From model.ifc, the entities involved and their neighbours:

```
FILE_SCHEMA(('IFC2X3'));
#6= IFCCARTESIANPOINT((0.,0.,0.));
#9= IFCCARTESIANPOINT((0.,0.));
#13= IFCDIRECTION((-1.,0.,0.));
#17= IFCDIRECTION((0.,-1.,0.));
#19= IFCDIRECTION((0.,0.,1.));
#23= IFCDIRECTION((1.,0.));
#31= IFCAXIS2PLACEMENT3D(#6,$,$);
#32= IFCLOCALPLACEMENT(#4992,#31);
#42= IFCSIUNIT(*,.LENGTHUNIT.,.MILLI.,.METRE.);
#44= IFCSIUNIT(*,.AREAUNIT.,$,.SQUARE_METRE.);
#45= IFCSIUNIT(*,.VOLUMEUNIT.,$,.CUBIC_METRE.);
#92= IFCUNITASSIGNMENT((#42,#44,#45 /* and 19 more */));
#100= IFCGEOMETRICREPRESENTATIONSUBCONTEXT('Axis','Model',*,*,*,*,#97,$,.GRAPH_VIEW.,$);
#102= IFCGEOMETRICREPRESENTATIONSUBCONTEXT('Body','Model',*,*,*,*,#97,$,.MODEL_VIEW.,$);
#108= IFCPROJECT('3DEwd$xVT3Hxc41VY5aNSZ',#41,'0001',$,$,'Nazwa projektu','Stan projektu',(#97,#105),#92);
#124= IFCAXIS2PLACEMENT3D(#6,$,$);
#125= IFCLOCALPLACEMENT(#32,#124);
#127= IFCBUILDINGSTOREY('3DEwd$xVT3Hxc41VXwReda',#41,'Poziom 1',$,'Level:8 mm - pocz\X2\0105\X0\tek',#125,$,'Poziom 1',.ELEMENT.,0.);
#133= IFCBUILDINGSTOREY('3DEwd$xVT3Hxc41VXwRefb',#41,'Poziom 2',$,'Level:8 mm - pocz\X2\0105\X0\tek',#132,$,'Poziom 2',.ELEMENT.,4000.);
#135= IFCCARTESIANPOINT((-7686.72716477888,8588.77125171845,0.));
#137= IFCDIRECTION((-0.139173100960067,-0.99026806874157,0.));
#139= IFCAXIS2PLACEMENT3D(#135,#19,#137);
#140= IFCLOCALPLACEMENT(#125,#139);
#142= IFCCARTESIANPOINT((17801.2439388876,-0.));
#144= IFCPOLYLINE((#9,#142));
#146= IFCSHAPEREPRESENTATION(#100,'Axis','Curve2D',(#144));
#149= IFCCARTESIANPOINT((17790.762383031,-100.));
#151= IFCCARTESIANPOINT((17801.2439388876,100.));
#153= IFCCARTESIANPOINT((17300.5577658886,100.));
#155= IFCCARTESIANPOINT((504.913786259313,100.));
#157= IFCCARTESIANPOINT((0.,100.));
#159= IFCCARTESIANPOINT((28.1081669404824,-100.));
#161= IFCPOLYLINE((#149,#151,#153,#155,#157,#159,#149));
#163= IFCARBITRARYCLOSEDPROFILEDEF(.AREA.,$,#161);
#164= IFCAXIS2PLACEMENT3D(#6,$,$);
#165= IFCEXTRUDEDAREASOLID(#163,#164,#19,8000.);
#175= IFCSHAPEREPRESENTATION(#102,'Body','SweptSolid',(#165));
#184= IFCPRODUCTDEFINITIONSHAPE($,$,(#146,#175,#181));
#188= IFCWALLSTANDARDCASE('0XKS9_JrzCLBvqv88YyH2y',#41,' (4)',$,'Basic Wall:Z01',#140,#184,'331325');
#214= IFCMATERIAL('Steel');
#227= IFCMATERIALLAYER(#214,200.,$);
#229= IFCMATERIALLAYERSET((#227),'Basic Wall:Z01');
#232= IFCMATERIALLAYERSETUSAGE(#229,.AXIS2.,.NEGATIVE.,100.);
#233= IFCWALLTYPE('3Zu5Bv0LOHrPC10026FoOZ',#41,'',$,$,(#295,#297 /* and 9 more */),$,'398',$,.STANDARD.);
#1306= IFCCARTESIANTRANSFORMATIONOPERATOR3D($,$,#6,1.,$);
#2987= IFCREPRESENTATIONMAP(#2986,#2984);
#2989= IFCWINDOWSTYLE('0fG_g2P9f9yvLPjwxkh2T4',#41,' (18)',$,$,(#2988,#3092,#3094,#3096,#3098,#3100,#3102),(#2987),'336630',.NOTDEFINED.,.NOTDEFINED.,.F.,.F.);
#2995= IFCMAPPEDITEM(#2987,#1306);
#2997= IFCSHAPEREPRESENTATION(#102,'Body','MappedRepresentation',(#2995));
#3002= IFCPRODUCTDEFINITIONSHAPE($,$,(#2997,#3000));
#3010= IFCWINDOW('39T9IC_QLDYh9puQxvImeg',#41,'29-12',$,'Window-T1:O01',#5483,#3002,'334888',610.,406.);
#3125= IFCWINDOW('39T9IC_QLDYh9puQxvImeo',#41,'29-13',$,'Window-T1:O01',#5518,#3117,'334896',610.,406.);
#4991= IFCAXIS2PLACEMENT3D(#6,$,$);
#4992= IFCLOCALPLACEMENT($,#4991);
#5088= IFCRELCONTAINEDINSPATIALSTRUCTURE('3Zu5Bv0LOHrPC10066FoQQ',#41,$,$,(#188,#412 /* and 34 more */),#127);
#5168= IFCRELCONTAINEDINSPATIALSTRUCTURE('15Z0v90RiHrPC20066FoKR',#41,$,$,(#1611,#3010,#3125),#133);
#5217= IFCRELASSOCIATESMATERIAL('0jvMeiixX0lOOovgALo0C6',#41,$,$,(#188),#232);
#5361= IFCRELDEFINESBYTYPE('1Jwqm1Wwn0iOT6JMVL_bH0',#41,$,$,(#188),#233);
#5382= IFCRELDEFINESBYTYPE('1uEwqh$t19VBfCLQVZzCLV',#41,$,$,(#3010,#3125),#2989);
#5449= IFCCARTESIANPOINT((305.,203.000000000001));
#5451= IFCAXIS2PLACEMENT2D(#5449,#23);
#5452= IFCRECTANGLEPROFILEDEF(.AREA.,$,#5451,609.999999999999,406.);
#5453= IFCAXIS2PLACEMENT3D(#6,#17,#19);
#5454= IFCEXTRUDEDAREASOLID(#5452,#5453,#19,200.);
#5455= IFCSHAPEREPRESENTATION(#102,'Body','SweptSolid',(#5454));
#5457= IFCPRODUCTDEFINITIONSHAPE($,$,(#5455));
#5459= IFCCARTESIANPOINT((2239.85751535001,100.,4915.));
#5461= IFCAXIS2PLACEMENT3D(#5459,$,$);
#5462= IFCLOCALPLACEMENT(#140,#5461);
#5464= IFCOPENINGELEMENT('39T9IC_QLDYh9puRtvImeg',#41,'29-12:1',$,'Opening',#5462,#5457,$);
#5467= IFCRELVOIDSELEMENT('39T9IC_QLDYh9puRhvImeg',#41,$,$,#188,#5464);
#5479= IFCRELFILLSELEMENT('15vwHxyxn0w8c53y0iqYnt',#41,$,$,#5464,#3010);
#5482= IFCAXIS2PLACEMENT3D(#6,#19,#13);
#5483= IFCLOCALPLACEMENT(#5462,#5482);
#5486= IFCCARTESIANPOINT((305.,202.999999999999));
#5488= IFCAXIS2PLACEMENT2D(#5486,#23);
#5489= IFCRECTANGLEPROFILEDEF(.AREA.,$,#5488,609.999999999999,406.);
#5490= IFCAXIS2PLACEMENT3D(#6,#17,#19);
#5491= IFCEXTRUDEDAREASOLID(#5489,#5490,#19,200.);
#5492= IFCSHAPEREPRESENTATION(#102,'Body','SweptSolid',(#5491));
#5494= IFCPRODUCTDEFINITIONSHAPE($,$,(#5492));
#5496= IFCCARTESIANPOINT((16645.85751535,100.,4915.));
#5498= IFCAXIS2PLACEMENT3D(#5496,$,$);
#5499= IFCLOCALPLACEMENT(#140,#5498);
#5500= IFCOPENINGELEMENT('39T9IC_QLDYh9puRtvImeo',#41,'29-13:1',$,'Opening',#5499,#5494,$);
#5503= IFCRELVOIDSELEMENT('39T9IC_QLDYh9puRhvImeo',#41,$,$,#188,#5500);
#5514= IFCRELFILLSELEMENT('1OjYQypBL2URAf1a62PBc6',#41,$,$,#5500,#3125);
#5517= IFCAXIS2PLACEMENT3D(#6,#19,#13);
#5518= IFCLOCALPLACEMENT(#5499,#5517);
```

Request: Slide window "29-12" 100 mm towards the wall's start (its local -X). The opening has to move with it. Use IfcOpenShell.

```python
import ifcopenshell
import ifcopenshell.api.geometry
import ifcopenshell.util.placement
import ifcopenshell.util.unit

model = ifcopenshell.open("model.ifc")
unit_scale = ifcopenshell.util.unit.calculate_unit_scale(model)

window = model.by_guid("39T9IC_QLDYh9puQxvImeg")
opening = window.FillsVoids[0].RelatingOpeningElement
wall = opening.VoidsElements[0].RelatingBuildingElement

wall_matrix = ifcopenshell.util.placement.get_local_placement(wall.ObjectPlacement)
shift = wall_matrix[:3, 0] * -0.1 / unit_scale
before = ifcopenshell.util.placement.get_local_placement(window.ObjectPlacement)[:3, 3].copy()

# The window is placed relative to its opening, so it follows when the opening moves.
matrix = ifcopenshell.util.placement.get_local_placement(opening.ObjectPlacement)
matrix[:3, 3] += shift
ifcopenshell.api.geometry.edit_object_placement(
    model, product=opening, matrix=matrix, is_si=False, should_transform_children=True
)

after = ifcopenshell.util.placement.get_local_placement(window.ObjectPlacement)[:3, 3]
print("window moved by", (after - before).round(3) + 0.0)

model.write("model_updated.ifc")
```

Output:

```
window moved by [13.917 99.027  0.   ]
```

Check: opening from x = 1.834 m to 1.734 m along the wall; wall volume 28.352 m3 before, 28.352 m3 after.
